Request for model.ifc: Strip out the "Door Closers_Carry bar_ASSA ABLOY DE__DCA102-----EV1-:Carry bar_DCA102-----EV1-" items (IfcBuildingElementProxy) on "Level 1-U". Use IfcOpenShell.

First a look at what the model holds.

```python
import ifcopenshell
import ifcopenshell.util.element

model = ifcopenshell.open("model.ifc")
print(model.schema)
storey = next(s for s in model.by_type("IfcBuildingStorey") if s.Name == "Level 1-U")
proxies = [e for e in ifcopenshell.util.element.get_decomposition(storey) if e.is_a("IfcBuildingElementProxy")]
seen = {}
for e in proxies:
    element_type = ifcopenshell.util.element.get_type(e)
    name = element_type.Name if element_type not in (None, e) else None
    seen[name] = seen.get(name, 0) + 1
for name, count in sorted(seen.items(), key=str):
    print(count, "x", name)
```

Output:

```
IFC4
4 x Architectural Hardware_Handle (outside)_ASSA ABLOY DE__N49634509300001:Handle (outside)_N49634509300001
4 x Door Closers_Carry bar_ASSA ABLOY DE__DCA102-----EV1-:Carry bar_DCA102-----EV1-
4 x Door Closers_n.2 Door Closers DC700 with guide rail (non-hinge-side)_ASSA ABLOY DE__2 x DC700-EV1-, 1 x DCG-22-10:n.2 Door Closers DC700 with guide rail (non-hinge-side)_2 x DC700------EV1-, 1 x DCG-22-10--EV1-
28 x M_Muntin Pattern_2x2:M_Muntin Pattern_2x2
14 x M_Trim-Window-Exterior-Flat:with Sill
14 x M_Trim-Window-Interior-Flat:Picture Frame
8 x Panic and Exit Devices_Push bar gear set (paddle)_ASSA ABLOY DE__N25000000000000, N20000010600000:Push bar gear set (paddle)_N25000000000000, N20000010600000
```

```python
import ifcopenshell
import ifcopenshell.api.root
import ifcopenshell.util.element

model = ifcopenshell.open("model.ifc")

storey = next(s for s in model.by_type("IfcBuildingStorey") if s.Name == "Level 1-U")
proxies = [e for e in ifcopenshell.util.element.get_decomposition(storey) if e.is_a("IfcBuildingElementProxy")]
targets = [e for e in proxies if (t := ifcopenshell.util.element.get_type(e)) not in (None, e) and t.Name == "Door Closers_Carry bar_ASSA ABLOY DE__DCA102-----EV1-:Carry bar_DCA102-----EV1-"]

for e in targets:
    ifcopenshell.api.root.remove_product(model, product=e)
print(len(targets), "removed")

model.write("model_v2.ifc")
```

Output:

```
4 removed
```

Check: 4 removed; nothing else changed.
